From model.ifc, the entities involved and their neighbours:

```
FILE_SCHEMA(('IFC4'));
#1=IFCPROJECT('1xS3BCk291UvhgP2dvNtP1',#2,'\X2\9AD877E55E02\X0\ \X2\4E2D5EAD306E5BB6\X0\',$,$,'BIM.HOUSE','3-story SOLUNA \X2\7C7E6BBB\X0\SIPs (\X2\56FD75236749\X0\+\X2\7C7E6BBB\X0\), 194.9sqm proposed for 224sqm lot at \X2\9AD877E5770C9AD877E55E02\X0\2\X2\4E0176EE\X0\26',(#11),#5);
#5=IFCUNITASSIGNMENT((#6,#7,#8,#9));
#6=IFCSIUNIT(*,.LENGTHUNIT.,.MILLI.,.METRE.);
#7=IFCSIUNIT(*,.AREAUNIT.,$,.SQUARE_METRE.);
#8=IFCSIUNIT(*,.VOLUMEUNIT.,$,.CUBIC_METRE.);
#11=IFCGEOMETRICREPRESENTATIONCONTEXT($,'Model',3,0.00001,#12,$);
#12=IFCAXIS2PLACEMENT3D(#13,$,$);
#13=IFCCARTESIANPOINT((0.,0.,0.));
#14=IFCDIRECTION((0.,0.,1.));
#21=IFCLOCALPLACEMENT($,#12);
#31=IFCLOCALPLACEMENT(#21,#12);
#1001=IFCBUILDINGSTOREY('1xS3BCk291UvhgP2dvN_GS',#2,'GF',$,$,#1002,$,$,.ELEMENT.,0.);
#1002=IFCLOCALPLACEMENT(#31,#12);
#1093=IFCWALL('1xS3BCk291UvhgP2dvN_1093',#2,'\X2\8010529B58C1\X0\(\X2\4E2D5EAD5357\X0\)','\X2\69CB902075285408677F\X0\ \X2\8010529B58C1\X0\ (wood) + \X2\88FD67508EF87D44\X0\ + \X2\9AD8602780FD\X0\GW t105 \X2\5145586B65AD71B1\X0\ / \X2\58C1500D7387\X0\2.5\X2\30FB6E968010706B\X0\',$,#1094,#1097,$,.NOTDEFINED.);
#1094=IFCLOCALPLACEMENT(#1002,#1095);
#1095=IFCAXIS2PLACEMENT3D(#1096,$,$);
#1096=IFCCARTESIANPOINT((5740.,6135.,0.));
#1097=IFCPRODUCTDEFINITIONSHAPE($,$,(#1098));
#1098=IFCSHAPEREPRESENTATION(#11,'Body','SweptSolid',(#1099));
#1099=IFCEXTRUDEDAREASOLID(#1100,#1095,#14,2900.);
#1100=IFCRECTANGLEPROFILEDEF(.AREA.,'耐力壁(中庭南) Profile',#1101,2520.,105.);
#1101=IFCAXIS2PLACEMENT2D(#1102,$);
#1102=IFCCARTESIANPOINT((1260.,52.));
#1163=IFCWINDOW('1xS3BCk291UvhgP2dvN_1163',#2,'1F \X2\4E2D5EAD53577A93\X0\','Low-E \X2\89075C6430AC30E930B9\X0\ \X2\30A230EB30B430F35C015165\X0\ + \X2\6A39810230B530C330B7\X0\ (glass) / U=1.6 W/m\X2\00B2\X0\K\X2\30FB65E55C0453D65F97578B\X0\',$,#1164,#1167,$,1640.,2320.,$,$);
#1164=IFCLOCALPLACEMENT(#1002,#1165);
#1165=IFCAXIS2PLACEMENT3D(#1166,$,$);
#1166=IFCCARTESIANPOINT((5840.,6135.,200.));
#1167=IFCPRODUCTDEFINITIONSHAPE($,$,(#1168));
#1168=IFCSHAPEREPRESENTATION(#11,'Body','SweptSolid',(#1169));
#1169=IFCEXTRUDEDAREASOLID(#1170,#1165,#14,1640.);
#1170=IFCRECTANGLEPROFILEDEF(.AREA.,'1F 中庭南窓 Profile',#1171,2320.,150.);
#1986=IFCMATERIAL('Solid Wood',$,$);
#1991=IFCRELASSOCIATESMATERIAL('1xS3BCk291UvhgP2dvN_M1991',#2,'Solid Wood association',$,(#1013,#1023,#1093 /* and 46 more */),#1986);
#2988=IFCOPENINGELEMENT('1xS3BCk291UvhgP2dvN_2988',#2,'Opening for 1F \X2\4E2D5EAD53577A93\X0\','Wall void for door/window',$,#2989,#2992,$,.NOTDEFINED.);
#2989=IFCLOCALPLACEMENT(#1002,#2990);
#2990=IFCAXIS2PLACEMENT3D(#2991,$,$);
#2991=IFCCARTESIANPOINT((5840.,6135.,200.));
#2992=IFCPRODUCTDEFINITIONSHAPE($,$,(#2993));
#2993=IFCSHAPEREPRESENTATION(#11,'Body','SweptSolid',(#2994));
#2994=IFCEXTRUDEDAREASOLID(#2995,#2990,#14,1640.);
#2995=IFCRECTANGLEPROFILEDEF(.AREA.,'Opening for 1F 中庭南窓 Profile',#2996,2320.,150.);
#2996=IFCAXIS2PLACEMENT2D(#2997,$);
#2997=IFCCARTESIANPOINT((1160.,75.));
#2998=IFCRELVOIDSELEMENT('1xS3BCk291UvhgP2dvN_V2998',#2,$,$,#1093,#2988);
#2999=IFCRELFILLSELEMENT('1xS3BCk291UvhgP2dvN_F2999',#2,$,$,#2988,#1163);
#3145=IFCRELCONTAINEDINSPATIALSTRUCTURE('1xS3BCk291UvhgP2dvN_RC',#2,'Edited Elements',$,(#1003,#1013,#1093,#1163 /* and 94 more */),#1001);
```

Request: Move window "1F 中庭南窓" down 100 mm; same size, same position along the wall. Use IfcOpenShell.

```python
import numpy as np
import ifcopenshell
import ifcopenshell.api.geometry
import ifcopenshell.util.placement
import ifcopenshell.util.unit

model = ifcopenshell.open("model.ifc")
unit_scale = ifcopenshell.util.unit.calculate_unit_scale(model)

window = model.by_guid("1xS3BCk291UvhgP2dvN_1163")
opening = window.FillsVoids[0].RelatingOpeningElement
dz = -0.1 / unit_scale

shift = np.array([0.0, 0.0, dz])
# The window is not placed relative to its opening, so move both.
for product in (opening, window):
    matrix = ifcopenshell.util.placement.get_local_placement(product.ObjectPlacement)
    matrix[:3, 3] += shift
    ifcopenshell.api.geometry.edit_object_placement(model, product=product, matrix=matrix, is_si=False)

print(f"moved by {dz * unit_scale:+.3f} m")

model.write("model-out.ifc")
```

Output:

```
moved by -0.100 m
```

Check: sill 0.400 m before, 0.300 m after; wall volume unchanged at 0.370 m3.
